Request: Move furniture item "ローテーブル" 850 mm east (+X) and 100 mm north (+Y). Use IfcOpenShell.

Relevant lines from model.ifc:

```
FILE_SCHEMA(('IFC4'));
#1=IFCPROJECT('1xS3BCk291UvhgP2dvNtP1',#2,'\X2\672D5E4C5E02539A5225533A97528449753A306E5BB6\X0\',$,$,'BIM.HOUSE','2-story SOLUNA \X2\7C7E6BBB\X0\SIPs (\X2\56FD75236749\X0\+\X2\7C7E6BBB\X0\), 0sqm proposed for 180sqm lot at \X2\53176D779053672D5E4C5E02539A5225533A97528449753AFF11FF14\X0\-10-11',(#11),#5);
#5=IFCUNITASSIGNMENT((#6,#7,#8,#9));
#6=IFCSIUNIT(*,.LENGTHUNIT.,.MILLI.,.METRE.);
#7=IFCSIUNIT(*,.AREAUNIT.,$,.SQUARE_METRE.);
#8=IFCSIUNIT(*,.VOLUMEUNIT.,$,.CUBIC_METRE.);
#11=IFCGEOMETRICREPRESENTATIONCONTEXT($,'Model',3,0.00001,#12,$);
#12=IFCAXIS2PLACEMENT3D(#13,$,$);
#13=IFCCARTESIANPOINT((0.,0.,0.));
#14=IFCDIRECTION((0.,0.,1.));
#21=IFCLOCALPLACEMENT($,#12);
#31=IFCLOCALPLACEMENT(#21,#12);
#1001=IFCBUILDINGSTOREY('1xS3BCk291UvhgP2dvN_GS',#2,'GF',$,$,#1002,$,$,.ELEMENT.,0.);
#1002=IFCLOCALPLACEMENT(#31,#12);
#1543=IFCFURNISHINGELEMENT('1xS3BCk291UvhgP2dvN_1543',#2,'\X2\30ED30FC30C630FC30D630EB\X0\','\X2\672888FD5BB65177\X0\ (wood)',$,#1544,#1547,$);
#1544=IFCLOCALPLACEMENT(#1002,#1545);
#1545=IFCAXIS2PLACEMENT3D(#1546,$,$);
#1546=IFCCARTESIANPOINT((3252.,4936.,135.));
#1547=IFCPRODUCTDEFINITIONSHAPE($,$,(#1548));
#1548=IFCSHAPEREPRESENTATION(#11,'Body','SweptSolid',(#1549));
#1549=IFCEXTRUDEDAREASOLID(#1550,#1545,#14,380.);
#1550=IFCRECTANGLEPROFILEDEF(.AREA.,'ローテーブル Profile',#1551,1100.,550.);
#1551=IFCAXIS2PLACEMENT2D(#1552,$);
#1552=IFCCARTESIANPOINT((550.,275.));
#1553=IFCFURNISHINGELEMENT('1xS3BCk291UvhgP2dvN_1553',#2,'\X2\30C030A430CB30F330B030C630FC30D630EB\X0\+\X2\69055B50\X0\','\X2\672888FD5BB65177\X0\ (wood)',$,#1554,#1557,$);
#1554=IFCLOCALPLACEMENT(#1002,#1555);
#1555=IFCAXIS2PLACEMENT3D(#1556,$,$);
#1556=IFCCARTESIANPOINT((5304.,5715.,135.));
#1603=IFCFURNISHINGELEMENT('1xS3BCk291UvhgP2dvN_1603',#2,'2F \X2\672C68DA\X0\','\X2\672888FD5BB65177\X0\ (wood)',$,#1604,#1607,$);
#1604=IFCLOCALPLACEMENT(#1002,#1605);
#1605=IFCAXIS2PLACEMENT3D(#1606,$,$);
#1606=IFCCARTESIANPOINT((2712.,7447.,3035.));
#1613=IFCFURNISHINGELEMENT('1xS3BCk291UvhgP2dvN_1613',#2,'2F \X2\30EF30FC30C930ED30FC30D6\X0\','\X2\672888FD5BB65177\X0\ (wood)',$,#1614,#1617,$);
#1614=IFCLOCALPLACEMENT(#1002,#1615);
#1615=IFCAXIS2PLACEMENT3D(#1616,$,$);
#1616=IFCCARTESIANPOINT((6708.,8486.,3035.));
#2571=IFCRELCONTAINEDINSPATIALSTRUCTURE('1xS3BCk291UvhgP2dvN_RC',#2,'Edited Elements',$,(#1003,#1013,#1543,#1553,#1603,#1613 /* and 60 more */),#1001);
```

```python
import ifcopenshell
import ifcopenshell.api.geometry
import ifcopenshell.util.placement
import ifcopenshell.util.unit

model = ifcopenshell.open("model.ifc")
unit_scale = ifcopenshell.util.unit.calculate_unit_scale(model)

item = model.by_guid("1xS3BCk291UvhgP2dvN_1543")
matrix = ifcopenshell.util.placement.get_local_placement(item.ObjectPlacement)
matrix[0, 3] += 0.85 / unit_scale
matrix[1, 3] += 0.1 / unit_scale
ifcopenshell.api.geometry.edit_object_placement(model, product=item, matrix=matrix, is_si=False)

print(ifcopenshell.util.placement.get_local_placement(item.ObjectPlacement).round(3) + 0.0)

model.write("model_edited.ifc")
```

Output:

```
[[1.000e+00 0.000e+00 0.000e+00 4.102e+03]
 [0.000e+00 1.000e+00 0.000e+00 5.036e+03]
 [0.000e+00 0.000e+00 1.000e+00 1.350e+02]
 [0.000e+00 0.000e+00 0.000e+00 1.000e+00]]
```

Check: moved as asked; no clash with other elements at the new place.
